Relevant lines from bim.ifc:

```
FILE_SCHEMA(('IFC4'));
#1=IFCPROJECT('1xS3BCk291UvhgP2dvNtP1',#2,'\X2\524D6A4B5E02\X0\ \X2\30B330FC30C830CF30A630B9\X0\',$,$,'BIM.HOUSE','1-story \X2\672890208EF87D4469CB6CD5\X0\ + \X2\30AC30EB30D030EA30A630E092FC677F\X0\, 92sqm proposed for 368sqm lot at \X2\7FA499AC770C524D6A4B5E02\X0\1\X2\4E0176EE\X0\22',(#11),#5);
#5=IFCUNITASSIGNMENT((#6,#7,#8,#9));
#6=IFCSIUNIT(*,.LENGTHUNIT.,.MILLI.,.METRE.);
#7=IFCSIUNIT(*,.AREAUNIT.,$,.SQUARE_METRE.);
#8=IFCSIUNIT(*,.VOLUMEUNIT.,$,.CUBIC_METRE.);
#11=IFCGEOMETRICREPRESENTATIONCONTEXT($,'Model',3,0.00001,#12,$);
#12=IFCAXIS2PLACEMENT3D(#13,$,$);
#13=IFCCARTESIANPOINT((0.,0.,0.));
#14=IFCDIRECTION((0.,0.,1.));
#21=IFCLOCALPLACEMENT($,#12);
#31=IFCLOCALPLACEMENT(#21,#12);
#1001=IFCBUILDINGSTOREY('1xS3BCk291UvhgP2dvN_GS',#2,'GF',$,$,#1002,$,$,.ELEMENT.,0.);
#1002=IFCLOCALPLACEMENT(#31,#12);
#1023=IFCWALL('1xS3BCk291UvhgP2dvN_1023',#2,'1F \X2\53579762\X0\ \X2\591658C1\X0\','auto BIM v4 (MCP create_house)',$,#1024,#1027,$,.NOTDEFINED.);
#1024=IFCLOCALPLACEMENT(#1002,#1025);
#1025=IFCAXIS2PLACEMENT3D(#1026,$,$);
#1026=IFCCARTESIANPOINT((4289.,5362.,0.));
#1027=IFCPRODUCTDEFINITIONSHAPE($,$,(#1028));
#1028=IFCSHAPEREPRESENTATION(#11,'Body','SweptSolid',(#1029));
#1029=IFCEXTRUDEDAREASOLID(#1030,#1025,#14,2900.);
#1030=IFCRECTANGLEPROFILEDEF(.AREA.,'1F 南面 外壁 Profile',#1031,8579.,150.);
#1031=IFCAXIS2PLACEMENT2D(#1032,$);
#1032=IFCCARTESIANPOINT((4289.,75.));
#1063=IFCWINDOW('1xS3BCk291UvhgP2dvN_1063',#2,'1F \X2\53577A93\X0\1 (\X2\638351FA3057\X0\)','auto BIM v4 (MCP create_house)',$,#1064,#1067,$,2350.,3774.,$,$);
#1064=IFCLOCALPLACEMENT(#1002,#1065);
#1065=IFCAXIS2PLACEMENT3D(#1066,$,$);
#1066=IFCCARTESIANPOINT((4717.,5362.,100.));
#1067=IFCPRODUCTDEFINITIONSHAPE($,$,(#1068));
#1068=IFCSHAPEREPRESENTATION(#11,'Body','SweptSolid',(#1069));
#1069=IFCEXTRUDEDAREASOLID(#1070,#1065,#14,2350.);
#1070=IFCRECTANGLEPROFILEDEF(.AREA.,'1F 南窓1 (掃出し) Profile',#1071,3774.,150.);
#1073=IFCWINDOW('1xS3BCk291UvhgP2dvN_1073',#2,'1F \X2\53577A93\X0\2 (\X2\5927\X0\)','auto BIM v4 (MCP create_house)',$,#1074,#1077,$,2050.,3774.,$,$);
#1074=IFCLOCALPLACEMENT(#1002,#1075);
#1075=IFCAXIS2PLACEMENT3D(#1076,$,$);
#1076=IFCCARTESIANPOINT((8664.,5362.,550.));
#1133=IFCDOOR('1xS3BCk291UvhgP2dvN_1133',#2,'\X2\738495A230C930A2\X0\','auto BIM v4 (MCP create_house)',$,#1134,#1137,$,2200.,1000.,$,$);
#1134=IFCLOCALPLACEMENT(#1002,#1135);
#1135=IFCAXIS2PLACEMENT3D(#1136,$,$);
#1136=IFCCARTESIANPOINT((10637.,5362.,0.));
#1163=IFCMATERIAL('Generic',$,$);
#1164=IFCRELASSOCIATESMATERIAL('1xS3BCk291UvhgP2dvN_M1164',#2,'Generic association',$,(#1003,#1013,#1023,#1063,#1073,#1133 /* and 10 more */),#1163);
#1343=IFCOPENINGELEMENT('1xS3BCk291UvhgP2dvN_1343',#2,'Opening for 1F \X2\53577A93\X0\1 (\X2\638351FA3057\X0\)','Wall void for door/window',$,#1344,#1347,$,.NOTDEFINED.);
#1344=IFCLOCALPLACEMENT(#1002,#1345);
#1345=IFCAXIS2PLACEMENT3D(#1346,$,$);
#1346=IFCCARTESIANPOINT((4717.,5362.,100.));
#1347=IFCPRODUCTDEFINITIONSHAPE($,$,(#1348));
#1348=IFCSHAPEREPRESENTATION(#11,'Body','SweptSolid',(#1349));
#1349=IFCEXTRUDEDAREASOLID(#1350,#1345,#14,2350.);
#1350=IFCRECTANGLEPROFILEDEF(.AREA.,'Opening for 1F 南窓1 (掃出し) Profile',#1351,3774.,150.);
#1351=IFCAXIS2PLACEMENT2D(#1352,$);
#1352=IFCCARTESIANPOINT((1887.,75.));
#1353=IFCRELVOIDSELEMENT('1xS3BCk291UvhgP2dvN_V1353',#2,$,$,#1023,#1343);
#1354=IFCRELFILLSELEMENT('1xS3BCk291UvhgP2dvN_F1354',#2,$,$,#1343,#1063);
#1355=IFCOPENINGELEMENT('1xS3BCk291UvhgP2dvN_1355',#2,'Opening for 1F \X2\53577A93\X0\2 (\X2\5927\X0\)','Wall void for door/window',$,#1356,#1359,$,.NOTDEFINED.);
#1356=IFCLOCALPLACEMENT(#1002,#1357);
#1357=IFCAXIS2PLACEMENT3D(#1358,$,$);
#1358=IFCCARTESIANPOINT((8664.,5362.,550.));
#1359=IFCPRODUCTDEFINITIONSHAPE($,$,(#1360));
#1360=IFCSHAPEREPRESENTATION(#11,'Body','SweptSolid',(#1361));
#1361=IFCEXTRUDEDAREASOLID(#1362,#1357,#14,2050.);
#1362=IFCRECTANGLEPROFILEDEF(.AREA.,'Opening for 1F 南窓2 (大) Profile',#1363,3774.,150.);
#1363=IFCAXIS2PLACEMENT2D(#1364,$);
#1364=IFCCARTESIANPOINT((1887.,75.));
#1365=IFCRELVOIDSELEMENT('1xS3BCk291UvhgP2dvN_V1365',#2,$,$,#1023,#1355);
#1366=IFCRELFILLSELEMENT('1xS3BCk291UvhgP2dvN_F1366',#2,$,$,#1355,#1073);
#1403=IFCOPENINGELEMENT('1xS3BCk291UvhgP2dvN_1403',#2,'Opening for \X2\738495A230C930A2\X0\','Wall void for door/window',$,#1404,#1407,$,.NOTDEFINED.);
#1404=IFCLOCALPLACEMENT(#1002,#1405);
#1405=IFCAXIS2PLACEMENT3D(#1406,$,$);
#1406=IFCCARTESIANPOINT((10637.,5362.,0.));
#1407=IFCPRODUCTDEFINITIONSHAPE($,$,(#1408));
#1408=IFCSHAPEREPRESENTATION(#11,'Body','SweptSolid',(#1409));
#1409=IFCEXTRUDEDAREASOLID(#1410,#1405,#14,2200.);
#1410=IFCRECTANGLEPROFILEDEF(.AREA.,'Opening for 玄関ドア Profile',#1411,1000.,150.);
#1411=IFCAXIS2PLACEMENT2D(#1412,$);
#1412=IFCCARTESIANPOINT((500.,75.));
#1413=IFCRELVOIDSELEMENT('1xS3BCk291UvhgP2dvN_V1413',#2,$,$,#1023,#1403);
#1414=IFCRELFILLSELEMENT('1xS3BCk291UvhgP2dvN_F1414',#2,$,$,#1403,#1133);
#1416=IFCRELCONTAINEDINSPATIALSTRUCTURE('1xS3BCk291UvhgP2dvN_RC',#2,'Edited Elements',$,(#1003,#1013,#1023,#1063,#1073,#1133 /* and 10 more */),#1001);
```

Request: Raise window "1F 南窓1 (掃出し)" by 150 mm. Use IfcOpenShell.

```python
import numpy as np
import ifcopenshell
import ifcopenshell.api.geometry
import ifcopenshell.util.placement
import ifcopenshell.util.unit

model = ifcopenshell.open("bim.ifc")
unit_scale = ifcopenshell.util.unit.calculate_unit_scale(model)

window = model.by_id(1063)
opening = window.FillsVoids[0].RelatingOpeningElement
dz = 0.15 / unit_scale

shift = np.array([0.0, 0.0, dz])
# The window is not placed relative to its opening, so move both.
for product in (opening, window):
    matrix = ifcopenshell.util.placement.get_local_placement(product.ObjectPlacement)
    matrix[:3, 3] += shift
    ifcopenshell.api.geometry.edit_object_placement(model, product=product, matrix=matrix, is_si=False)

print(f"moved by {dz * unit_scale:+.3f} m")

model.write("bim_updated.ifc")
```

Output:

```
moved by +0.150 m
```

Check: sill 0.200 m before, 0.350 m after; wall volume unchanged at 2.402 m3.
